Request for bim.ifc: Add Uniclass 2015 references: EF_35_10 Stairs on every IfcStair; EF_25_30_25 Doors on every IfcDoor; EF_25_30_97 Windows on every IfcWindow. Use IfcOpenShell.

First a look at what the model holds.

```python
import ifcopenshell

model = ifcopenshell.open("bim.ifc")
print(model.schema)
print("classifications:", [c.Name for c in model.by_type("IfcClassification")])
for ifc_class in ("IfcDoor", "IfcRoof", "IfcStair", "IfcWall", "IfcWindow"):
    print(ifc_class, len(model.by_type(ifc_class)))
```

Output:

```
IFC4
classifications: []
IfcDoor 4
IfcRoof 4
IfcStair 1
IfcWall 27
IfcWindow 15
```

```python
import ifcopenshell
import ifcopenshell.api.classification

model = ifcopenshell.open("bim.ifc")

system = ifcopenshell.api.classification.add_classification(model, classification="Uniclass 2015")

codes = {
    "IfcStair": ("EF_35_10", "Stairs"),
    "IfcDoor": ("EF_25_30_25", "Doors"),
    "IfcWindow": ("EF_25_30_97", "Windows"),
}
for ifc_class, (code, name) in codes.items():
    products = model.by_type(ifc_class)
    ifcopenshell.api.classification.add_reference(
        model, products=products, classification=system, identification=code, name=name
    )
    print(code, len(products))

model.write("bim-out.ifc")
```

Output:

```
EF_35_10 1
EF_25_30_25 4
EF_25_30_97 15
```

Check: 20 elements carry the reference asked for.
